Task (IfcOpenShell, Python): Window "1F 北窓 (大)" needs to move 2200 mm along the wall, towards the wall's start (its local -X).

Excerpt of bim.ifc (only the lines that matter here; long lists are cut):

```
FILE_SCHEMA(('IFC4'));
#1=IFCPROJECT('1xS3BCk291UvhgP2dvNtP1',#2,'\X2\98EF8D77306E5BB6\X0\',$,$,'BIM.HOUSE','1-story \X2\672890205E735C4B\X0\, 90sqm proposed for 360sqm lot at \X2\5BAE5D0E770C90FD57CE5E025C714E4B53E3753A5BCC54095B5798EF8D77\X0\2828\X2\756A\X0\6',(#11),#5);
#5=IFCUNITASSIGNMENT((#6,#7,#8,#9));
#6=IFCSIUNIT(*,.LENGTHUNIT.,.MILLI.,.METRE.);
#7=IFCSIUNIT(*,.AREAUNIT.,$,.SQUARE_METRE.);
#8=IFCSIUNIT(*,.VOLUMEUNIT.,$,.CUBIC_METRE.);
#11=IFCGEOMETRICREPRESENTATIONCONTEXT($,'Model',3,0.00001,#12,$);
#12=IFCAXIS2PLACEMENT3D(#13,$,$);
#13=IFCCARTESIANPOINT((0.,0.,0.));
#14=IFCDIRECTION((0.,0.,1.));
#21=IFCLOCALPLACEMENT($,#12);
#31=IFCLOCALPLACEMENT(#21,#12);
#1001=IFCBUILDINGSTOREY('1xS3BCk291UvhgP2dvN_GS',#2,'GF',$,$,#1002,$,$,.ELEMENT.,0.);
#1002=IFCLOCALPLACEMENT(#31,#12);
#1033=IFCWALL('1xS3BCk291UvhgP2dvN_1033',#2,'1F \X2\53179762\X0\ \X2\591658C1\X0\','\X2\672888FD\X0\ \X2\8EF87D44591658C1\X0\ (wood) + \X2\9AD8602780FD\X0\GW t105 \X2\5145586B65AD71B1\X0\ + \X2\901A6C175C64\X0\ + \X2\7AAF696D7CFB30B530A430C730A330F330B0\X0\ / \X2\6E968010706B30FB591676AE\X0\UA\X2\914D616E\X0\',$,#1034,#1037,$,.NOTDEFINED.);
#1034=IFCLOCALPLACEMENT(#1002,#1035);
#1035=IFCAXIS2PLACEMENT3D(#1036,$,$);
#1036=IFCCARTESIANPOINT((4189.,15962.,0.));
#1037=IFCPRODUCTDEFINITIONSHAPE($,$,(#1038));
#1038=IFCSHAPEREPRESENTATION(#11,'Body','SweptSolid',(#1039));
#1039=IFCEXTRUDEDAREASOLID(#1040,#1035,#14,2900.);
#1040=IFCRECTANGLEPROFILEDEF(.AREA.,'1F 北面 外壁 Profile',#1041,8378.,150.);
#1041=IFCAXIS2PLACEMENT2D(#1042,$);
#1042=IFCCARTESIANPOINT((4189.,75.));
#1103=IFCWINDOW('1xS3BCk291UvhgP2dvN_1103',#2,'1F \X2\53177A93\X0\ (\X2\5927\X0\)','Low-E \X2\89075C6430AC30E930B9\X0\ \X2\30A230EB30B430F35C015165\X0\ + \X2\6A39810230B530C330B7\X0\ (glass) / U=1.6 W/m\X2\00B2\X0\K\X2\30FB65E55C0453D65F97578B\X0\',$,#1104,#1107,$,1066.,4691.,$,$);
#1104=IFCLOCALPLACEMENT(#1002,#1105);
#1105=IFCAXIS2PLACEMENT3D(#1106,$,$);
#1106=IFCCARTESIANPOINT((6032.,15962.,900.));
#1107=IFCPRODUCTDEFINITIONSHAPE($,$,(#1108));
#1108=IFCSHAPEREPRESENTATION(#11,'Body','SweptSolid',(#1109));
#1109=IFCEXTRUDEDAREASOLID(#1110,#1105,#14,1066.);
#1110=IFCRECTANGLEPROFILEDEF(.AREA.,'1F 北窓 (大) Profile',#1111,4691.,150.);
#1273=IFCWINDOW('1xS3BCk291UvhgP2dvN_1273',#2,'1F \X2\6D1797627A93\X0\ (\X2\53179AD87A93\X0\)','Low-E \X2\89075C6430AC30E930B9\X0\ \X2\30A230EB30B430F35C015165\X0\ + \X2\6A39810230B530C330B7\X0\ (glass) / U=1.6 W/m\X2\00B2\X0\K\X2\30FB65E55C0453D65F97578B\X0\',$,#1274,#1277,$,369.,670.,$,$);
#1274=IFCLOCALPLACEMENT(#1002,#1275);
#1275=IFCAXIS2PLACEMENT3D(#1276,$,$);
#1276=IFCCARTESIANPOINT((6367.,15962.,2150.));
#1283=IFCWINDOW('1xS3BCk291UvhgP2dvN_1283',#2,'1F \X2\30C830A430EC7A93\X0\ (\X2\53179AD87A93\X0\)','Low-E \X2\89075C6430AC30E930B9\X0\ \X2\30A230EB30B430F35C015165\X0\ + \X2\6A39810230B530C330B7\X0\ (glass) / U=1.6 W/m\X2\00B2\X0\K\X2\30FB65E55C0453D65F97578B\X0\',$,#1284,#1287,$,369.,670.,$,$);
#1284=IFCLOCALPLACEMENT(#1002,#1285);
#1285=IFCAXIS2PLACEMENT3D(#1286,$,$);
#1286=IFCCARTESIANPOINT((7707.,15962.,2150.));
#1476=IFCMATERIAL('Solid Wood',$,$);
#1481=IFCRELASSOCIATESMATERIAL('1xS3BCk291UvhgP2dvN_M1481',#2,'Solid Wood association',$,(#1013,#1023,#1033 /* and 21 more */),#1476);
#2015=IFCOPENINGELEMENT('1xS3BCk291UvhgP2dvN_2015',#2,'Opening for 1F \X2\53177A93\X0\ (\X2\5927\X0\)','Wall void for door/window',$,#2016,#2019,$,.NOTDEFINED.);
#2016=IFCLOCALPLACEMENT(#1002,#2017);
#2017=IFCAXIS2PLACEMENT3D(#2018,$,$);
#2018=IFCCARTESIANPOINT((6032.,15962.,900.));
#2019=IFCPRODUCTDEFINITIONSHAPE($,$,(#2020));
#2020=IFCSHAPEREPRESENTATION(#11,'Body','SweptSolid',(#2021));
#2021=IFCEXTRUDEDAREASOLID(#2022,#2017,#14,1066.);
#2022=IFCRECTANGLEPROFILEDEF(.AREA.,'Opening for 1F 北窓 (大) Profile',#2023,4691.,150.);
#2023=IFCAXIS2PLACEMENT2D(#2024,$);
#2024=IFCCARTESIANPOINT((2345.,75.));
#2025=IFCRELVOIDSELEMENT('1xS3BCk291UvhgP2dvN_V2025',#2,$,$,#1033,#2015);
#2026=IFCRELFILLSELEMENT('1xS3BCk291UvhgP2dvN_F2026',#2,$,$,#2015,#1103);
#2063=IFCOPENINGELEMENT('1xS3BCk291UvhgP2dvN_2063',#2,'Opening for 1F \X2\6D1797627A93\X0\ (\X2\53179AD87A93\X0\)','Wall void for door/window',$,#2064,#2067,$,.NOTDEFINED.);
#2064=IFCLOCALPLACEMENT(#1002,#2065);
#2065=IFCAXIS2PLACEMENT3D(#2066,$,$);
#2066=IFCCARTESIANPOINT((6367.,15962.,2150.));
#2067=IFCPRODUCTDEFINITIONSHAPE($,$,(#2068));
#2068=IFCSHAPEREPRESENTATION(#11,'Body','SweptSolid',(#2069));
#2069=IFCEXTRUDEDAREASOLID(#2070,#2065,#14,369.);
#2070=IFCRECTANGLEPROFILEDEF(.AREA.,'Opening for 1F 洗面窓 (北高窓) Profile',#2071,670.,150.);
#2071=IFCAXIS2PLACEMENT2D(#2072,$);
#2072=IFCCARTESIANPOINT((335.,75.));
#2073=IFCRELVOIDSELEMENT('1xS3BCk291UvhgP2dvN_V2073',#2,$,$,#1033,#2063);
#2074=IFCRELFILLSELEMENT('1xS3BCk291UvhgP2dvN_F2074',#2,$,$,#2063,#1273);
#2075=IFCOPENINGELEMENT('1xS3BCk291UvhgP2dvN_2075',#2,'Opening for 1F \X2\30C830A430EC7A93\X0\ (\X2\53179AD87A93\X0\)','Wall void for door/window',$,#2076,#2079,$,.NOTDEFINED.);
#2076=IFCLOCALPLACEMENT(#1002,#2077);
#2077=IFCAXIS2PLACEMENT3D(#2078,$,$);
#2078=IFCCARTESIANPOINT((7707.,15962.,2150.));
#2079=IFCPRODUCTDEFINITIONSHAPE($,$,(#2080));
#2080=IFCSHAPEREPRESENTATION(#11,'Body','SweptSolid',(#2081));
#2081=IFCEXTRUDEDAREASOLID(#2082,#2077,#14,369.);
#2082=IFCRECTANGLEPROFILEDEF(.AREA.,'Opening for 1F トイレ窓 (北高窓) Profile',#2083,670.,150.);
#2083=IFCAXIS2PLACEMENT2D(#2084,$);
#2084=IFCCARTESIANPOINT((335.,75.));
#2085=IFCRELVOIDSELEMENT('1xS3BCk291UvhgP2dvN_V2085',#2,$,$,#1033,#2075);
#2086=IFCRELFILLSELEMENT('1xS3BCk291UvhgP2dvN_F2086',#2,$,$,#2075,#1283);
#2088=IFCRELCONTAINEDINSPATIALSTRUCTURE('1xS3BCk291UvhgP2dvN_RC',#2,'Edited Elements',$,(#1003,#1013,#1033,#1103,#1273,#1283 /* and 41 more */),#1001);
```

```python
import ifcopenshell
import ifcopenshell.api.geometry
import ifcopenshell.util.placement
import ifcopenshell.util.unit

model = ifcopenshell.open("bim.ifc")
unit_scale = ifcopenshell.util.unit.calculate_unit_scale(model)

window = model.by_guid("1xS3BCk291UvhgP2dvN_1103")
opening = window.FillsVoids[0].RelatingOpeningElement
wall = opening.VoidsElements[0].RelatingBuildingElement

wall_matrix = ifcopenshell.util.placement.get_local_placement(wall.ObjectPlacement)
shift = wall_matrix[:3, 0] * -2.2 / unit_scale
before = ifcopenshell.util.placement.get_local_placement(window.ObjectPlacement)[:3, 3].copy()

# The window is not placed relative to its opening, so move both.
for product in (opening, window):
    matrix = ifcopenshell.util.placement.get_local_placement(product.ObjectPlacement)
    matrix[:3, 3] += shift
    ifcopenshell.api.geometry.edit_object_placement(model, product=product, matrix=matrix, is_si=False)

after = ifcopenshell.util.placement.get_local_placement(window.ObjectPlacement)[:3, 3]
print("window moved by", (after - before).round(3) + 0.0)

model.write("bim_rev.ifc")
```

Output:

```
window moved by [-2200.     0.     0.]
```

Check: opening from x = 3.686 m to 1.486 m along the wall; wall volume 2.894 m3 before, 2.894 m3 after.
